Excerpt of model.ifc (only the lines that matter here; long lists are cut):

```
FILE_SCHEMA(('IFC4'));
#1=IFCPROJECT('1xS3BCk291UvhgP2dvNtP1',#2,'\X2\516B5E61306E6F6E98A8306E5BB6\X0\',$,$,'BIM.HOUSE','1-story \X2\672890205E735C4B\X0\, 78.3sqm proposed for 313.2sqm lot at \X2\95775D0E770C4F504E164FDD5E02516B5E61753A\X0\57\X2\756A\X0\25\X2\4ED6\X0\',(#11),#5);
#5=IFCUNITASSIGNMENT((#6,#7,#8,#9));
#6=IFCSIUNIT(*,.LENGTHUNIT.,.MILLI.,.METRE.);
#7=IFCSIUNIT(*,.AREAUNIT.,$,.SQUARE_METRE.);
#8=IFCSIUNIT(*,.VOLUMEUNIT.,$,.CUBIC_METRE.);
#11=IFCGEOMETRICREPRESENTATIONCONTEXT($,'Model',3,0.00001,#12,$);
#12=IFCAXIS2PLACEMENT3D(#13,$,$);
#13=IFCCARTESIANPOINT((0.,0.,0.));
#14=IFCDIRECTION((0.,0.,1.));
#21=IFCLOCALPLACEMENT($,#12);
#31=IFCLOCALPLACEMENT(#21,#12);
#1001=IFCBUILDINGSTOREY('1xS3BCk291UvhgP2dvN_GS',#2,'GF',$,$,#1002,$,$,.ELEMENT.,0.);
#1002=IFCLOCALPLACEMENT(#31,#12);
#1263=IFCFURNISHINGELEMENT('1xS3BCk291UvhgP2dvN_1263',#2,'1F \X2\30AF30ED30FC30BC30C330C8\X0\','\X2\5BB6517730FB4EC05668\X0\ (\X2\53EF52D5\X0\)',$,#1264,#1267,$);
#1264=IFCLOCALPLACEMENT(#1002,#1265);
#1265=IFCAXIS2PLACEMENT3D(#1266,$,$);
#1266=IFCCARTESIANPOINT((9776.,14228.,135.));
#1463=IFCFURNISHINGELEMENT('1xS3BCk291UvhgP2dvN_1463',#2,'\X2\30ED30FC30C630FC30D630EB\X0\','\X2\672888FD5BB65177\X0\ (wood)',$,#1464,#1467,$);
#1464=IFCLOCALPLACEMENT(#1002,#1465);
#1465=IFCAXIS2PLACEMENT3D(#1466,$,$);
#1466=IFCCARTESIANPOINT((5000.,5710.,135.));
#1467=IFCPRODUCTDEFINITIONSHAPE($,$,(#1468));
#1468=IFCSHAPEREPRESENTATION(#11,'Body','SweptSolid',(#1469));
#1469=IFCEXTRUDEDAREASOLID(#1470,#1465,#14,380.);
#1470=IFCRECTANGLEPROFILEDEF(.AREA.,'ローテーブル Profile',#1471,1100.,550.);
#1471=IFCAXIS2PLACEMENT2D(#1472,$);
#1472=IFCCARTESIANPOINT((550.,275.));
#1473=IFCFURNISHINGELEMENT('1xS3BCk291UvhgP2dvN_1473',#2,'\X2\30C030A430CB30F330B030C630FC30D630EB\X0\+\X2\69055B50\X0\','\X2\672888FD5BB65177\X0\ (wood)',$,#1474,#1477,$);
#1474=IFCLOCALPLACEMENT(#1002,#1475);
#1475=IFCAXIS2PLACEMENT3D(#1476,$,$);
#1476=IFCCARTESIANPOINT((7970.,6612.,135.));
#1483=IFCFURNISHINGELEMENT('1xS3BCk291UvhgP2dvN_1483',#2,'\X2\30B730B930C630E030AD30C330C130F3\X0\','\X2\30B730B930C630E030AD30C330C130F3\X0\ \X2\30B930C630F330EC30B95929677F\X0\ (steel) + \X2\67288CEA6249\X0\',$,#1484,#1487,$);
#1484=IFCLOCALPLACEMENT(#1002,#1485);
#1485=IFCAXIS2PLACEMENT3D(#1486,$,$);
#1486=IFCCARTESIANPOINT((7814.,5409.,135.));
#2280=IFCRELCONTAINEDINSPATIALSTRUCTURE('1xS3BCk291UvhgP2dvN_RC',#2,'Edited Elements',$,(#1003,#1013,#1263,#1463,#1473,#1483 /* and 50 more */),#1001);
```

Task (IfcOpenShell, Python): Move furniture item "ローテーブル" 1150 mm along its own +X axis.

```python
import ifcopenshell
import ifcopenshell.api.geometry
import ifcopenshell.util.placement
import ifcopenshell.util.unit

model = ifcopenshell.open("model.ifc")
unit_scale = ifcopenshell.util.unit.calculate_unit_scale(model)

item = model.by_guid("1xS3BCk291UvhgP2dvN_1463")
matrix = ifcopenshell.util.placement.get_local_placement(item.ObjectPlacement)
matrix[:3, 3] += matrix[:3, 0] * 1.15 / unit_scale
ifcopenshell.api.geometry.edit_object_placement(model, product=item, matrix=matrix, is_si=False)

print(ifcopenshell.util.placement.get_local_placement(item.ObjectPlacement).round(3) + 0.0)

model.write("model_edited.ifc")
```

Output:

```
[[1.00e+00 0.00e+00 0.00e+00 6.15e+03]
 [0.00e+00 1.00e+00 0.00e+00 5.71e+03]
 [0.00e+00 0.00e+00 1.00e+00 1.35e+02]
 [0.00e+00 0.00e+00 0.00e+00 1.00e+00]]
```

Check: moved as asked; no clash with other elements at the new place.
